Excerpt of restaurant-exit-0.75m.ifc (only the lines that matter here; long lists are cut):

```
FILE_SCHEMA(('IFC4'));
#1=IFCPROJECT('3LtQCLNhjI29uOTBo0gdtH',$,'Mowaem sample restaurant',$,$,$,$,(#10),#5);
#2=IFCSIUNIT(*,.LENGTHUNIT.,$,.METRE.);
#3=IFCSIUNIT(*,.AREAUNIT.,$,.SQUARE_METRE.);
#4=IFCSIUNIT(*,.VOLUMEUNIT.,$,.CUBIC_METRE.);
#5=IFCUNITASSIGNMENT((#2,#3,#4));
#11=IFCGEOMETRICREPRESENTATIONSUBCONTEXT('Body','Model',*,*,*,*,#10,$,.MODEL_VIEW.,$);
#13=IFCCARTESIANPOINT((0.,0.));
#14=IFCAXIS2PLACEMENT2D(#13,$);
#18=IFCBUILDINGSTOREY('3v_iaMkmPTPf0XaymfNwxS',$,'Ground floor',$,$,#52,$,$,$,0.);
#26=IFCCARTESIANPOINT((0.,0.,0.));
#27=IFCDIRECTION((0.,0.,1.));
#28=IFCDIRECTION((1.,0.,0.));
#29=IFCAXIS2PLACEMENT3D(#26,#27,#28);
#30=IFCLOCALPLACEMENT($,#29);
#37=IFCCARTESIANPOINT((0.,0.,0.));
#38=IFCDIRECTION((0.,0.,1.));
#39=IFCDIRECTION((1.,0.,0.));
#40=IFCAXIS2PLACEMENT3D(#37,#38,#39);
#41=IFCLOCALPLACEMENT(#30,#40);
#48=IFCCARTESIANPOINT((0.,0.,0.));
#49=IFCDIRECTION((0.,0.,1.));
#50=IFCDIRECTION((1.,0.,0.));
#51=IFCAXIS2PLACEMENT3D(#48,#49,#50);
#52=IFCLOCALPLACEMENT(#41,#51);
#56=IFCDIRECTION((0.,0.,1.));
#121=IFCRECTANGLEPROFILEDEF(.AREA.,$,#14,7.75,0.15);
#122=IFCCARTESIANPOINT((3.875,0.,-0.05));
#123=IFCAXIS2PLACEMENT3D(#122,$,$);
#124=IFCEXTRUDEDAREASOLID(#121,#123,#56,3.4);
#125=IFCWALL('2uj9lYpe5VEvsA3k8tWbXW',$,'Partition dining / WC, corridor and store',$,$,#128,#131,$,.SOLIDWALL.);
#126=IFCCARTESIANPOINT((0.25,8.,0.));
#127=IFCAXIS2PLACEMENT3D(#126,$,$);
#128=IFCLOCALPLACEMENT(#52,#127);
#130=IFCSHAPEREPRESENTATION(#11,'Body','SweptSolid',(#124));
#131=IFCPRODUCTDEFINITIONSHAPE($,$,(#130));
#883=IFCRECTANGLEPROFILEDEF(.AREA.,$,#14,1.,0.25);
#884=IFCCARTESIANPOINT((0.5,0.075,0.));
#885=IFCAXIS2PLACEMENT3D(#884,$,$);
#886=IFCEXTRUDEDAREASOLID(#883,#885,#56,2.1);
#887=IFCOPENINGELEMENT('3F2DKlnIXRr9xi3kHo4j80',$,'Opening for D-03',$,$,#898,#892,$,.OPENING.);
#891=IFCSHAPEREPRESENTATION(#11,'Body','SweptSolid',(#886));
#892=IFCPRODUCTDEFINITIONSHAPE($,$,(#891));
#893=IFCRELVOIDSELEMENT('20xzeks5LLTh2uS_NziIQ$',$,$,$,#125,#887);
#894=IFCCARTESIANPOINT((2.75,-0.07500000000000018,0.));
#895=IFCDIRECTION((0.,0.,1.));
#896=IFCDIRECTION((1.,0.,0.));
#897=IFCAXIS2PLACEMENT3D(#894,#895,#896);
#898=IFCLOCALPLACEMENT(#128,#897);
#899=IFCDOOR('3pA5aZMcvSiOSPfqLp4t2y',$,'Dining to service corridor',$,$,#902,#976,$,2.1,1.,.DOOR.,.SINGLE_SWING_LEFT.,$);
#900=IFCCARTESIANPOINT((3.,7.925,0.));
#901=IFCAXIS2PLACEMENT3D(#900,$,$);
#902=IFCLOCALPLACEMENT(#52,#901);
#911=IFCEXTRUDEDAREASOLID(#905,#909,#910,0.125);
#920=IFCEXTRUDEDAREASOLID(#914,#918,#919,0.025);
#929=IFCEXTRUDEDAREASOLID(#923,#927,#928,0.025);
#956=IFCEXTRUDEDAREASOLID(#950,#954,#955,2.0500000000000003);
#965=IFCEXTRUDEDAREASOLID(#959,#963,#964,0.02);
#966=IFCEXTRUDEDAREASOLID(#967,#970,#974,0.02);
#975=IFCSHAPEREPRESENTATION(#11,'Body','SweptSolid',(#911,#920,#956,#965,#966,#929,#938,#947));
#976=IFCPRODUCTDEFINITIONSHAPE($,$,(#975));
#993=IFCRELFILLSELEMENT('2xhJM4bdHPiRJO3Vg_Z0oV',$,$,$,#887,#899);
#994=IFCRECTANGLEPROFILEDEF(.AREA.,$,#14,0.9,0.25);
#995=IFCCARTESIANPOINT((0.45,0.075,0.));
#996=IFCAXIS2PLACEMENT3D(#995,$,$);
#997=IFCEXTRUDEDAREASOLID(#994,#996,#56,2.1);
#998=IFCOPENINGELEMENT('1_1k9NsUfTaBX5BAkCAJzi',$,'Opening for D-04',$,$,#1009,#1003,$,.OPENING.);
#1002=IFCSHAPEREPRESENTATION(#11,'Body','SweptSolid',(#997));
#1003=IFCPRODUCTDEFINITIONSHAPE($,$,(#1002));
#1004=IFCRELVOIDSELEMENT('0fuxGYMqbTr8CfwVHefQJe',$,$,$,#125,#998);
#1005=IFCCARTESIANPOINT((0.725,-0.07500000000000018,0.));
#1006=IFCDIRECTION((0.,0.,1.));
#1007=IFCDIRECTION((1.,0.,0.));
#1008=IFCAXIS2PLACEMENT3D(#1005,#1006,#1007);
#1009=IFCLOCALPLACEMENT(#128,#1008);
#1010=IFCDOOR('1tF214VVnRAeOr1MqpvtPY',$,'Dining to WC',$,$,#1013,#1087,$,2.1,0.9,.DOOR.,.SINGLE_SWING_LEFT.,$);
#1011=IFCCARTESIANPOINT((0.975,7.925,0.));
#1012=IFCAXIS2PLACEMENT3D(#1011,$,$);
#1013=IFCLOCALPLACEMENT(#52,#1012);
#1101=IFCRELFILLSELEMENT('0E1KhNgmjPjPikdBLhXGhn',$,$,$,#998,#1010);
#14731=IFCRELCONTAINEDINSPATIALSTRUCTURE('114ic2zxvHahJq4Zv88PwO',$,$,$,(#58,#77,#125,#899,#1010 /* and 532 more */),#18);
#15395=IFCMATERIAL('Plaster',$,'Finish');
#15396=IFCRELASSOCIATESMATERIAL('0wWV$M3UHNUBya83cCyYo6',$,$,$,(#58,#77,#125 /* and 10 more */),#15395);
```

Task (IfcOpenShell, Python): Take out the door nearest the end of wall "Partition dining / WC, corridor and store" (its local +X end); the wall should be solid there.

```python
import ifcopenshell
import ifcopenshell.api.feature
import ifcopenshell.api.root
import ifcopenshell.geom
import ifcopenshell.util.shape

model = ifcopenshell.open("restaurant-exit-0.75m.ifc")
settings = ifcopenshell.geom.settings()


def volume(element):
    """Net volume in cubic metres, openings subtracted."""
    shape = ifcopenshell.geom.create_shape(settings, element)
    return ifcopenshell.util.shape.get_volume(shape.geometry)


door = model.by_guid("3pA5aZMcvSiOSPfqLp4t2y")
opening = door.FillsVoids[0].RelatingOpeningElement
wall = opening.VoidsElements[0].RelatingBuildingElement
before = volume(wall)

ifcopenshell.api.root.remove_product(model, product=door)
ifcopenshell.api.feature.remove_feature(model, feature=opening)

after = volume(wall)

print(f"wall volume {before:.3f} -> {after:.3f} m3")

model.write("restaurant-exit-0.75m_edited.ifc")
```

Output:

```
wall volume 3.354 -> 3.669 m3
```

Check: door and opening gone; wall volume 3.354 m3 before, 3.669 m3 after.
